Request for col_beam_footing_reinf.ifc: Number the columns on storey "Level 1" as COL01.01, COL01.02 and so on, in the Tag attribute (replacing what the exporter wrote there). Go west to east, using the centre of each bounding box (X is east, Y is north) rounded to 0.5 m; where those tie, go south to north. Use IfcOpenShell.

First a look at what the model holds.

```python
import ifcopenshell
import ifcopenshell.util.element
import ifcopenshell.util.placement

model = ifcopenshell.open("col_beam_footing_reinf.ifc")
print(model.schema)
storey = next(s for s in model.by_type("IfcBuildingStorey") if s.Name == "Level 1")
columns = [e for e in ifcopenshell.util.element.get_decomposition(storey) if e.is_a("IfcColumn")]
for e in sorted(columns, key=lambda e: e.id()):
    origin = ifcopenshell.util.placement.get_local_placement(e.ObjectPlacement)[:3, 3]
    print(e.id(), e.Tag, e.Name, origin.round(2) + 0.0, sep=" | ")
```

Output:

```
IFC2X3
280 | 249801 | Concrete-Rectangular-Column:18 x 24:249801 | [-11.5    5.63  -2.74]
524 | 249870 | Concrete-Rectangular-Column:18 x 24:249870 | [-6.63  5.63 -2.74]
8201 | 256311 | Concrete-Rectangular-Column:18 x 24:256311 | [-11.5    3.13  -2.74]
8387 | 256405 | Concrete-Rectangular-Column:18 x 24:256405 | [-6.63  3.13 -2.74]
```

```python
import ifcopenshell
import ifcopenshell.geom
import ifcopenshell.util.element
import ifcopenshell.util.shape

model = ifcopenshell.open("col_beam_footing_reinf.ifc")
settings = ifcopenshell.geom.settings()
settings.set("use-world-coords", True)


def centre(element):
    shape = ifcopenshell.geom.create_shape(settings, element)
    return ifcopenshell.util.shape.get_bbox_centroid(shape.geometry)


storey = next(s for s in model.by_type("IfcBuildingStorey") if s.Name == "Level 1")
columns = [e for e in ifcopenshell.util.element.get_decomposition(storey) if e.is_a("IfcColumn")]

# Insertion points can sit at a corner or the storey origin, so sort by the geometry (in metres).
centres = {e: centre(e) for e in columns}
columns.sort(key=lambda e: (round(centres[e][0] / 0.5), centres[e][1]))

for i, e in enumerate(columns, start=1):
    number = f"COL01.{i:02d}"
    e.Tag = number
    print(e.id(), number)

model.write("col_beam_footing_reinf_rev.ifc")
```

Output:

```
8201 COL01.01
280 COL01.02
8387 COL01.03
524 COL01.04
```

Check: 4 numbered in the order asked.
